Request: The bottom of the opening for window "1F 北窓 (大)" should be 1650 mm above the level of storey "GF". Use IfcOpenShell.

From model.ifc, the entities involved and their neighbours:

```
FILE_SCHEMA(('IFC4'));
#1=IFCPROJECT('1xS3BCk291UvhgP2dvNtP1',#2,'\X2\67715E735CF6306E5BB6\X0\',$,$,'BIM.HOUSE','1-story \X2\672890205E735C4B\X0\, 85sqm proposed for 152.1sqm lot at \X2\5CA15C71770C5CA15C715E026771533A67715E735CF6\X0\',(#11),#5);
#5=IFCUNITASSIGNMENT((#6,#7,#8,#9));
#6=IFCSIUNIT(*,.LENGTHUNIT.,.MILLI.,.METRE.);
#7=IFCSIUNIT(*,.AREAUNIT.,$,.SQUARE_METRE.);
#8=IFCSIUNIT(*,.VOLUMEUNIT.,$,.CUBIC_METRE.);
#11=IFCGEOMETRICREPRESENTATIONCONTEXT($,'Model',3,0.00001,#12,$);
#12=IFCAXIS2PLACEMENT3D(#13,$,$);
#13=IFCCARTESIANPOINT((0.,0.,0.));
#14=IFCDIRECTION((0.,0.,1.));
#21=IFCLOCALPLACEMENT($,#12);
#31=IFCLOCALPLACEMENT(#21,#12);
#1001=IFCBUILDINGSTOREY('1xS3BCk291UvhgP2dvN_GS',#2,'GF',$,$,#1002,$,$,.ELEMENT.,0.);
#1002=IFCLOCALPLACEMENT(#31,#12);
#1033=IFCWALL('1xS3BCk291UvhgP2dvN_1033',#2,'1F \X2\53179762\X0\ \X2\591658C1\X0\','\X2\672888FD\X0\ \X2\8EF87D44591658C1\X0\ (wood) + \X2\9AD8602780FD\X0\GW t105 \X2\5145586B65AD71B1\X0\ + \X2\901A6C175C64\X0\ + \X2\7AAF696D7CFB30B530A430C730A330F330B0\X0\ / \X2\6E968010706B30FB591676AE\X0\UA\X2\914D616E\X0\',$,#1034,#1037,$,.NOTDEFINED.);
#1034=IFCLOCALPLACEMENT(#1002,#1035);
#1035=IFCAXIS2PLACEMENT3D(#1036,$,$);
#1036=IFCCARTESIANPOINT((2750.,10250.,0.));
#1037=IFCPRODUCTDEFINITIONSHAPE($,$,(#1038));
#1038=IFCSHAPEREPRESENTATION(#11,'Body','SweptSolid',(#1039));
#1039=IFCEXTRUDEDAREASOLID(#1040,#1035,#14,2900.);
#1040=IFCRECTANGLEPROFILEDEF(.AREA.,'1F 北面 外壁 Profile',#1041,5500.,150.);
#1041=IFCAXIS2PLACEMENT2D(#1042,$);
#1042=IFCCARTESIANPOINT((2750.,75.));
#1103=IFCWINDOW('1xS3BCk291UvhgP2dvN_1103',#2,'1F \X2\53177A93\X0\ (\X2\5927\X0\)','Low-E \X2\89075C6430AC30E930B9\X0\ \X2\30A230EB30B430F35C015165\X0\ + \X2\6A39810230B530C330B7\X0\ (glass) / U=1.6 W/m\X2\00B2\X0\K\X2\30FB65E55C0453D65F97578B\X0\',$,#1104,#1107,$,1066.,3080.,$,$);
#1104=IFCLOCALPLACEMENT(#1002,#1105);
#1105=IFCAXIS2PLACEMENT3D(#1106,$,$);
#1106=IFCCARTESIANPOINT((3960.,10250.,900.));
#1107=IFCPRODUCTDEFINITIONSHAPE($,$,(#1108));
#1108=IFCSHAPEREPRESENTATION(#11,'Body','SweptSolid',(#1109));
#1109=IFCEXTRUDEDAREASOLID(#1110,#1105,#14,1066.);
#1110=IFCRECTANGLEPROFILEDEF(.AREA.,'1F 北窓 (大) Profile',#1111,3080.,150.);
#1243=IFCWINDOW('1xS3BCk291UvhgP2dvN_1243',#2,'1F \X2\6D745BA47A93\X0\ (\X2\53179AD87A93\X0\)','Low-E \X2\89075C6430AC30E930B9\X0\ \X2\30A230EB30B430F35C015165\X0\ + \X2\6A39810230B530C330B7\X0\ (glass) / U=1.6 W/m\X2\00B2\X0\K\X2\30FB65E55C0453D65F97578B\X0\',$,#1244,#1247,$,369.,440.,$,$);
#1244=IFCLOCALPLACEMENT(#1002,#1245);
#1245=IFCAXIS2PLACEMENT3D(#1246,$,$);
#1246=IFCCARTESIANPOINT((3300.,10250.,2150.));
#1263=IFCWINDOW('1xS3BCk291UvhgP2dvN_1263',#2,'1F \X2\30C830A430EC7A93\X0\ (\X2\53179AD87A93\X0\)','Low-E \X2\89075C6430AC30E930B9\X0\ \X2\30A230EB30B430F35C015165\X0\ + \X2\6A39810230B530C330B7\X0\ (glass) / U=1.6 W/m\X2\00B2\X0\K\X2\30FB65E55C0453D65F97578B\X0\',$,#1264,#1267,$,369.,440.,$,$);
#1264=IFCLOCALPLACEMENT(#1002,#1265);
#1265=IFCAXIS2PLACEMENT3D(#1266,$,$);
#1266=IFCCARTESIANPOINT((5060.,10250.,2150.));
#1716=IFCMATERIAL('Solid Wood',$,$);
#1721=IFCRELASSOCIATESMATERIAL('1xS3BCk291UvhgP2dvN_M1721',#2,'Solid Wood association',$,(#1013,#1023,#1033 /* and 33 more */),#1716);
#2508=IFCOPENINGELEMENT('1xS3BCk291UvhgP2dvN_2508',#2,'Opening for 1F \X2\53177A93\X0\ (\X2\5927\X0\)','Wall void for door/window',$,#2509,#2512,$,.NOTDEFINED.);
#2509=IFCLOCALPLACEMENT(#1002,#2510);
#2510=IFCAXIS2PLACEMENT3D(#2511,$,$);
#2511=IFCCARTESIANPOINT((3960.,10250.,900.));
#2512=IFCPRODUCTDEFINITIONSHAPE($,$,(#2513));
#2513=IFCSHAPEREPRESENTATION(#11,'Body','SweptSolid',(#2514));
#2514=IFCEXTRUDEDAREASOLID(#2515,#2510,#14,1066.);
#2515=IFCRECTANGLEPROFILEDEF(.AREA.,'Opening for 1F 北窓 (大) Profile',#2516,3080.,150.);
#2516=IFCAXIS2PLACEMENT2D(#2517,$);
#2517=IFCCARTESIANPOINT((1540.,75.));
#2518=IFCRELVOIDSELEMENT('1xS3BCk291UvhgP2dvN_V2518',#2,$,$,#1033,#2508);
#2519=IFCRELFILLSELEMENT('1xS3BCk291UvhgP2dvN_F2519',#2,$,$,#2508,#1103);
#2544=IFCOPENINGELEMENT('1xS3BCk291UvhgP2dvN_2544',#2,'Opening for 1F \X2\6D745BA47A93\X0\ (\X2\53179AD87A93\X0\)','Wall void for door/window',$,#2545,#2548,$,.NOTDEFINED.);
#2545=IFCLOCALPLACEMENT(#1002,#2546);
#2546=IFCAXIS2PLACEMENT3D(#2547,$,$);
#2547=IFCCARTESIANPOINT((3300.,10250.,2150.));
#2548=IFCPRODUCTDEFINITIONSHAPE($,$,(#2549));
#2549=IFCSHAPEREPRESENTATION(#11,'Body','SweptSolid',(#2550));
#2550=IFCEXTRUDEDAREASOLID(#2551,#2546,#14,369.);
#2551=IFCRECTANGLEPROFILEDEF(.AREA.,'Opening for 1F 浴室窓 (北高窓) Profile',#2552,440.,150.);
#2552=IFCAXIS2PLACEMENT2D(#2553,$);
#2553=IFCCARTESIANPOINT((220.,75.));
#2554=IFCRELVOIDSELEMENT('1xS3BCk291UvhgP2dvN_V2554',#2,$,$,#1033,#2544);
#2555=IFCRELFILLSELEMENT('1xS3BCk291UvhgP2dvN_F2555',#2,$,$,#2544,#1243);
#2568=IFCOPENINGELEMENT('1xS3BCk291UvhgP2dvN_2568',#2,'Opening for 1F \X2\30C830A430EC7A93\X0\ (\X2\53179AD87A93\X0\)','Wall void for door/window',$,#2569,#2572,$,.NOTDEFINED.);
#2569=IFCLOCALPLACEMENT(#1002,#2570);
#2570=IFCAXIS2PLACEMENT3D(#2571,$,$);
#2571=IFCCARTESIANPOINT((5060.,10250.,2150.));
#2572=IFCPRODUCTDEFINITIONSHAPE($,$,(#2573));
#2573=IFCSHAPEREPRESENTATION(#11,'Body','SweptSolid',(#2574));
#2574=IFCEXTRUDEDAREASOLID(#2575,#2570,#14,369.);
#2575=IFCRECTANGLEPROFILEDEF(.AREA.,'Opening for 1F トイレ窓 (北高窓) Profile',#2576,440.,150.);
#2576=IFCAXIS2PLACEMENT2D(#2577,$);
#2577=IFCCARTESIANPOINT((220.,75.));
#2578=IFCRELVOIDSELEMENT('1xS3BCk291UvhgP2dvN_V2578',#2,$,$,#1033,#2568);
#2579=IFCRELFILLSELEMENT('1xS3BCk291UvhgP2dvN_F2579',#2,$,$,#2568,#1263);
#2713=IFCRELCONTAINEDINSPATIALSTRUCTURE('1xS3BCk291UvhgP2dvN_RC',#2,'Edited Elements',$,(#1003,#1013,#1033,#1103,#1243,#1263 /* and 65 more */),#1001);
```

```python
import numpy as np
import ifcopenshell
import ifcopenshell.api.geometry
import ifcopenshell.geom
import ifcopenshell.util.element
import ifcopenshell.util.placement
import ifcopenshell.util.shape
import ifcopenshell.util.unit

model = ifcopenshell.open("model.ifc")
unit_scale = ifcopenshell.util.unit.calculate_unit_scale(model)

window = model.by_guid("1xS3BCk291UvhgP2dvN_1103")
opening = window.FillsVoids[0].RelatingOpeningElement
storey = ifcopenshell.util.element.get_container(window, ifc_class="IfcBuildingStorey")
level = ifcopenshell.util.placement.get_local_placement(storey.ObjectPlacement)[2, 3]

# The opening's origin need not be at the sill, so measure its lowest point.
shape = ifcopenshell.geom.create_shape(ifcopenshell.geom.settings(), opening)
bottom = ifcopenshell.util.shape.get_shape_bottom_elevation(shape, shape.geometry) / unit_scale
dz = level + 1.65 / unit_scale - bottom

shift = np.array([0.0, 0.0, dz])
# The window is not placed relative to its opening, so move both.
for product in (opening, window):
    matrix = ifcopenshell.util.placement.get_local_placement(product.ObjectPlacement)
    matrix[:3, 3] += shift
    ifcopenshell.api.geometry.edit_object_placement(model, product=product, matrix=matrix, is_si=False)

print(f"moved by {dz * unit_scale:+.3f} m")

model.write("model_rev.ifc")
```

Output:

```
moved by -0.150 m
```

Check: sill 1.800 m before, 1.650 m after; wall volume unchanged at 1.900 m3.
